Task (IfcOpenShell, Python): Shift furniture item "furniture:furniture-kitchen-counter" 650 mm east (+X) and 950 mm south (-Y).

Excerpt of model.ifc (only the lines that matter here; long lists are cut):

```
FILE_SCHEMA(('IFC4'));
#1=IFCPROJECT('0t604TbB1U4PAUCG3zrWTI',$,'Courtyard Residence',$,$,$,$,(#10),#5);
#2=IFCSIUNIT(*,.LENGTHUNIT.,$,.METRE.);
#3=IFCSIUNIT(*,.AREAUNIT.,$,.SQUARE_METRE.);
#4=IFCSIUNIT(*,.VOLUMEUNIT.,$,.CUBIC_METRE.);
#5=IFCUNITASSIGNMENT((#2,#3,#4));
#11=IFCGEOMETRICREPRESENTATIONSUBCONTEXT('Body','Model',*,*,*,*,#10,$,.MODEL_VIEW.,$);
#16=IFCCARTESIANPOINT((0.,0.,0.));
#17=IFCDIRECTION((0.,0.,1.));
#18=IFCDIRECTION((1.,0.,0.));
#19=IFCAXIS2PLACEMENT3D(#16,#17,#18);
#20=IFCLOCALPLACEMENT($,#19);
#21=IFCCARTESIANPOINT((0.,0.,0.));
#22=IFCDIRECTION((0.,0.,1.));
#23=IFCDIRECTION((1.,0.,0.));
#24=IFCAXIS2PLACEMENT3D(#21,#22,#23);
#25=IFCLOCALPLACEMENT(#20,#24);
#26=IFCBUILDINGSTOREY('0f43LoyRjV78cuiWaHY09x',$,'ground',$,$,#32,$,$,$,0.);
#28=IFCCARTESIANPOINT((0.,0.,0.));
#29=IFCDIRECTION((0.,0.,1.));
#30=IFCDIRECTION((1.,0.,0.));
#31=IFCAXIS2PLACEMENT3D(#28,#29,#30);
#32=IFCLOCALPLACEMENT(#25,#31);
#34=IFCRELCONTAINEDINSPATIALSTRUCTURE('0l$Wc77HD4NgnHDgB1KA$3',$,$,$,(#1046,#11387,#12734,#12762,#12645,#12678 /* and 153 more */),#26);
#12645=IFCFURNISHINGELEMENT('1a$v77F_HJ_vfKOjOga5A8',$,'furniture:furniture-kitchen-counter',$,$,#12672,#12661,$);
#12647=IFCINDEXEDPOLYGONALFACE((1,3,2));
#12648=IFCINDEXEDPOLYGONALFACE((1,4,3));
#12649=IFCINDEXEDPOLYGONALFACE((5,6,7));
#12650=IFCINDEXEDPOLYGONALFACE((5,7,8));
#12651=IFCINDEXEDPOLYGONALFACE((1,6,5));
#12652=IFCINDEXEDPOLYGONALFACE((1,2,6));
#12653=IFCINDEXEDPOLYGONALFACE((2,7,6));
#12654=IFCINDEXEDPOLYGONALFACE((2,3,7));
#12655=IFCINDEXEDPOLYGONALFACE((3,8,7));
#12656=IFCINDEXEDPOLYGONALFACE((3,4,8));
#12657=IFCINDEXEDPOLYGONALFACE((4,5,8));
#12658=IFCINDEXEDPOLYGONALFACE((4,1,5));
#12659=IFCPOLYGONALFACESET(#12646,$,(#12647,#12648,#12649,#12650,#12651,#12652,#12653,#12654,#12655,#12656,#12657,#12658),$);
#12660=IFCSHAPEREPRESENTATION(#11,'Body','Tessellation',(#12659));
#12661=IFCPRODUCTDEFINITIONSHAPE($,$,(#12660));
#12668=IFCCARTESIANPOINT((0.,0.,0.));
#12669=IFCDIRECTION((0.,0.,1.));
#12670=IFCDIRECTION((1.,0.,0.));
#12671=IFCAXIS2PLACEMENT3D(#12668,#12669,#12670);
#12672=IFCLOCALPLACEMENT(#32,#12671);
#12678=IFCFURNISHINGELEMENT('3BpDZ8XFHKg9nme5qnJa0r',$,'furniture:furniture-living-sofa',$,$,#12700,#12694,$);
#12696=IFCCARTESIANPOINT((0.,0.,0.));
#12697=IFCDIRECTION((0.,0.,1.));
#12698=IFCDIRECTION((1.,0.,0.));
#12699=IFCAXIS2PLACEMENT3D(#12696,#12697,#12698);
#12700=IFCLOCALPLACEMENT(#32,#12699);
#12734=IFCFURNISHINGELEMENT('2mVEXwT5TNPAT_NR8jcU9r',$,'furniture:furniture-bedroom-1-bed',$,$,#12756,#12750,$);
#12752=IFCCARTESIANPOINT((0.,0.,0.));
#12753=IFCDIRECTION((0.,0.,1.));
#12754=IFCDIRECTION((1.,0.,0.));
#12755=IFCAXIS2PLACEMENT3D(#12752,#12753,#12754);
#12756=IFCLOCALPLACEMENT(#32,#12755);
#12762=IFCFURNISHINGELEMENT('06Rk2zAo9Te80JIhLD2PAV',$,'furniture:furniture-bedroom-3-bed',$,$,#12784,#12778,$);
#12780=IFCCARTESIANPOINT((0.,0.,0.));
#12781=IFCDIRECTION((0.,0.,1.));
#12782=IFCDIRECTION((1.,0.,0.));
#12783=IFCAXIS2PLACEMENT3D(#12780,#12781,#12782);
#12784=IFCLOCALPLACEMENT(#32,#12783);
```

```python
import ifcopenshell
import ifcopenshell.api.geometry
import ifcopenshell.util.placement
import ifcopenshell.util.unit

model = ifcopenshell.open("model.ifc")
unit_scale = ifcopenshell.util.unit.calculate_unit_scale(model)

item = model.by_guid("1a$v77F_HJ_vfKOjOga5A8")
matrix = ifcopenshell.util.placement.get_local_placement(item.ObjectPlacement)
matrix[0, 3] += 0.65 / unit_scale
matrix[1, 3] -= 0.95 / unit_scale
ifcopenshell.api.geometry.edit_object_placement(model, product=item, matrix=matrix, is_si=False)

print(ifcopenshell.util.placement.get_local_placement(item.ObjectPlacement).round(3) + 0.0)

model.write("model_updated.ifc")
```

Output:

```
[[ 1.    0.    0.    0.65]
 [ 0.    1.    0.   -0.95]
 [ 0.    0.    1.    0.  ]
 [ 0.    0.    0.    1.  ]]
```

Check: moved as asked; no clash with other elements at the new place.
